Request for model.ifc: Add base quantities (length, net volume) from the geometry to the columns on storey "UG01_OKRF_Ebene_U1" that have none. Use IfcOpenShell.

First a look at what the model holds.

```python
import ifcopenshell
import ifcopenshell.util.element
import ifcopenshell.util.unit

model = ifcopenshell.open("model.ifc")
print(model.schema)
for unit_type in ("LENGTHUNIT", "AREAUNIT", "VOLUMEUNIT"):
    print(unit_type, ifcopenshell.util.unit.calculate_unit_scale(model, unit_type))
storey = next(s for s in model.by_type("IfcBuildingStorey") if s.Name == "UG01_OKRF_Ebene_U1")
columns = [e for e in ifcopenshell.util.element.get_decomposition(storey) if e.is_a("IfcColumn")]
for e in sorted(columns, key=lambda e: e.id()):
    print(e.id(), e.is_a(), e.Name, list(ifcopenshell.util.element.get_psets(e, qtos_only=True)), sep=" | ")
```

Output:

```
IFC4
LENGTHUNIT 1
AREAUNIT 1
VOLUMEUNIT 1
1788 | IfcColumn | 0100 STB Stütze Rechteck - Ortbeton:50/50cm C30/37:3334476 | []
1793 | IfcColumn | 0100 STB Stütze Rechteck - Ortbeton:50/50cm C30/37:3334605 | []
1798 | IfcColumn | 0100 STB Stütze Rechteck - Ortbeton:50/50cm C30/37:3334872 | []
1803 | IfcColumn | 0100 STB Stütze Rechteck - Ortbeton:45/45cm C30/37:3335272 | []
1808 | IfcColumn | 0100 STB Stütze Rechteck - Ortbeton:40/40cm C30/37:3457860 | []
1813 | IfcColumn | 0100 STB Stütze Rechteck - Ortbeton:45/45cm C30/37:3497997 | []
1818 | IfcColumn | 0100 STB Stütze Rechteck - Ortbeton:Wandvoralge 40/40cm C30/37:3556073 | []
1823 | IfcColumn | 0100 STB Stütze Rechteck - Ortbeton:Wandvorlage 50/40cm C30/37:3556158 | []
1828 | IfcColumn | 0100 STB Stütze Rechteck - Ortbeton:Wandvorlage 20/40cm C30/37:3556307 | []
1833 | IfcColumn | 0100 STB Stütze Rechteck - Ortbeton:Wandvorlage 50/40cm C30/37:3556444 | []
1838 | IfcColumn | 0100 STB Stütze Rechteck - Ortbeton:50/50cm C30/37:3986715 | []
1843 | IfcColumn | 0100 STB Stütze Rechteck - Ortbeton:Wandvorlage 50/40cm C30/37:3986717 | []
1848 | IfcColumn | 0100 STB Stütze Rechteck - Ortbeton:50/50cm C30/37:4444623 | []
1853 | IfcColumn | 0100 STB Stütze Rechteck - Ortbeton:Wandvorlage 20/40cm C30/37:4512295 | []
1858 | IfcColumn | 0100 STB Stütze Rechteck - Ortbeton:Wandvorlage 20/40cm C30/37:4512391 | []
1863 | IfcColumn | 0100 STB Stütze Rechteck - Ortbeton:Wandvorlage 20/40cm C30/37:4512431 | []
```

```python
import ifcopenshell
import ifcopenshell.api.pset
import ifcopenshell.geom
import ifcopenshell.util.element
import ifcopenshell.util.shape
import ifcopenshell.util.unit

model = ifcopenshell.open("model.ifc")
unit_scale = ifcopenshell.util.unit.calculate_unit_scale(model)
volume_scale = ifcopenshell.util.unit.calculate_unit_scale(model, "VOLUMEUNIT")
settings = ifcopenshell.geom.settings()

storey = next(s for s in model.by_type("IfcBuildingStorey") if s.Name == "UG01_OKRF_Ebene_U1")
columns = [e for e in ifcopenshell.util.element.get_decomposition(storey) if e.is_a("IfcColumn")]

for e in sorted(columns, key=lambda e: e.id()):
    if ifcopenshell.util.element.get_psets(e, qtos_only=True, should_inherit=False):
        continue
    # Geometry comes back in metres, in the element's own axes.
    shape = ifcopenshell.geom.create_shape(settings, e)
    values = {
        "Length": ifcopenshell.util.shape.get_z(shape.geometry) / unit_scale,
        "NetVolume": ifcopenshell.util.shape.get_volume(shape.geometry) / volume_scale,
    }
    qto = ifcopenshell.api.pset.add_qto(model, product=e, name="Qto_ColumnBaseQuantities")
    ifcopenshell.api.pset.edit_qto(model, qto=qto, properties=values)
    print(e.id(), {k: round(v, 3) for k, v in values.items()})

model.write("model_v2.ifc")
```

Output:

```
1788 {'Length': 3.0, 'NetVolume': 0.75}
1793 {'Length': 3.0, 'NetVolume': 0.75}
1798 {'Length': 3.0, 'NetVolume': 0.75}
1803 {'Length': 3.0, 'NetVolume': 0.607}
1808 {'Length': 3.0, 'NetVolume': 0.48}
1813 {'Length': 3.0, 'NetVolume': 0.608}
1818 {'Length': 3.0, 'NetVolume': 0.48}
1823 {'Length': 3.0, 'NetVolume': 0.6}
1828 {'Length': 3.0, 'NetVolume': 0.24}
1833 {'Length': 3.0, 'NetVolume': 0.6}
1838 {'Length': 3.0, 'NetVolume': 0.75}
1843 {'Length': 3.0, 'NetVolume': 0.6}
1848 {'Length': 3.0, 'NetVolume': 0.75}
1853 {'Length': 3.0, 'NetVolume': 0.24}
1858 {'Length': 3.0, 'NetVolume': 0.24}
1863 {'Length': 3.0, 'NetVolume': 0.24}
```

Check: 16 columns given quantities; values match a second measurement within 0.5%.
